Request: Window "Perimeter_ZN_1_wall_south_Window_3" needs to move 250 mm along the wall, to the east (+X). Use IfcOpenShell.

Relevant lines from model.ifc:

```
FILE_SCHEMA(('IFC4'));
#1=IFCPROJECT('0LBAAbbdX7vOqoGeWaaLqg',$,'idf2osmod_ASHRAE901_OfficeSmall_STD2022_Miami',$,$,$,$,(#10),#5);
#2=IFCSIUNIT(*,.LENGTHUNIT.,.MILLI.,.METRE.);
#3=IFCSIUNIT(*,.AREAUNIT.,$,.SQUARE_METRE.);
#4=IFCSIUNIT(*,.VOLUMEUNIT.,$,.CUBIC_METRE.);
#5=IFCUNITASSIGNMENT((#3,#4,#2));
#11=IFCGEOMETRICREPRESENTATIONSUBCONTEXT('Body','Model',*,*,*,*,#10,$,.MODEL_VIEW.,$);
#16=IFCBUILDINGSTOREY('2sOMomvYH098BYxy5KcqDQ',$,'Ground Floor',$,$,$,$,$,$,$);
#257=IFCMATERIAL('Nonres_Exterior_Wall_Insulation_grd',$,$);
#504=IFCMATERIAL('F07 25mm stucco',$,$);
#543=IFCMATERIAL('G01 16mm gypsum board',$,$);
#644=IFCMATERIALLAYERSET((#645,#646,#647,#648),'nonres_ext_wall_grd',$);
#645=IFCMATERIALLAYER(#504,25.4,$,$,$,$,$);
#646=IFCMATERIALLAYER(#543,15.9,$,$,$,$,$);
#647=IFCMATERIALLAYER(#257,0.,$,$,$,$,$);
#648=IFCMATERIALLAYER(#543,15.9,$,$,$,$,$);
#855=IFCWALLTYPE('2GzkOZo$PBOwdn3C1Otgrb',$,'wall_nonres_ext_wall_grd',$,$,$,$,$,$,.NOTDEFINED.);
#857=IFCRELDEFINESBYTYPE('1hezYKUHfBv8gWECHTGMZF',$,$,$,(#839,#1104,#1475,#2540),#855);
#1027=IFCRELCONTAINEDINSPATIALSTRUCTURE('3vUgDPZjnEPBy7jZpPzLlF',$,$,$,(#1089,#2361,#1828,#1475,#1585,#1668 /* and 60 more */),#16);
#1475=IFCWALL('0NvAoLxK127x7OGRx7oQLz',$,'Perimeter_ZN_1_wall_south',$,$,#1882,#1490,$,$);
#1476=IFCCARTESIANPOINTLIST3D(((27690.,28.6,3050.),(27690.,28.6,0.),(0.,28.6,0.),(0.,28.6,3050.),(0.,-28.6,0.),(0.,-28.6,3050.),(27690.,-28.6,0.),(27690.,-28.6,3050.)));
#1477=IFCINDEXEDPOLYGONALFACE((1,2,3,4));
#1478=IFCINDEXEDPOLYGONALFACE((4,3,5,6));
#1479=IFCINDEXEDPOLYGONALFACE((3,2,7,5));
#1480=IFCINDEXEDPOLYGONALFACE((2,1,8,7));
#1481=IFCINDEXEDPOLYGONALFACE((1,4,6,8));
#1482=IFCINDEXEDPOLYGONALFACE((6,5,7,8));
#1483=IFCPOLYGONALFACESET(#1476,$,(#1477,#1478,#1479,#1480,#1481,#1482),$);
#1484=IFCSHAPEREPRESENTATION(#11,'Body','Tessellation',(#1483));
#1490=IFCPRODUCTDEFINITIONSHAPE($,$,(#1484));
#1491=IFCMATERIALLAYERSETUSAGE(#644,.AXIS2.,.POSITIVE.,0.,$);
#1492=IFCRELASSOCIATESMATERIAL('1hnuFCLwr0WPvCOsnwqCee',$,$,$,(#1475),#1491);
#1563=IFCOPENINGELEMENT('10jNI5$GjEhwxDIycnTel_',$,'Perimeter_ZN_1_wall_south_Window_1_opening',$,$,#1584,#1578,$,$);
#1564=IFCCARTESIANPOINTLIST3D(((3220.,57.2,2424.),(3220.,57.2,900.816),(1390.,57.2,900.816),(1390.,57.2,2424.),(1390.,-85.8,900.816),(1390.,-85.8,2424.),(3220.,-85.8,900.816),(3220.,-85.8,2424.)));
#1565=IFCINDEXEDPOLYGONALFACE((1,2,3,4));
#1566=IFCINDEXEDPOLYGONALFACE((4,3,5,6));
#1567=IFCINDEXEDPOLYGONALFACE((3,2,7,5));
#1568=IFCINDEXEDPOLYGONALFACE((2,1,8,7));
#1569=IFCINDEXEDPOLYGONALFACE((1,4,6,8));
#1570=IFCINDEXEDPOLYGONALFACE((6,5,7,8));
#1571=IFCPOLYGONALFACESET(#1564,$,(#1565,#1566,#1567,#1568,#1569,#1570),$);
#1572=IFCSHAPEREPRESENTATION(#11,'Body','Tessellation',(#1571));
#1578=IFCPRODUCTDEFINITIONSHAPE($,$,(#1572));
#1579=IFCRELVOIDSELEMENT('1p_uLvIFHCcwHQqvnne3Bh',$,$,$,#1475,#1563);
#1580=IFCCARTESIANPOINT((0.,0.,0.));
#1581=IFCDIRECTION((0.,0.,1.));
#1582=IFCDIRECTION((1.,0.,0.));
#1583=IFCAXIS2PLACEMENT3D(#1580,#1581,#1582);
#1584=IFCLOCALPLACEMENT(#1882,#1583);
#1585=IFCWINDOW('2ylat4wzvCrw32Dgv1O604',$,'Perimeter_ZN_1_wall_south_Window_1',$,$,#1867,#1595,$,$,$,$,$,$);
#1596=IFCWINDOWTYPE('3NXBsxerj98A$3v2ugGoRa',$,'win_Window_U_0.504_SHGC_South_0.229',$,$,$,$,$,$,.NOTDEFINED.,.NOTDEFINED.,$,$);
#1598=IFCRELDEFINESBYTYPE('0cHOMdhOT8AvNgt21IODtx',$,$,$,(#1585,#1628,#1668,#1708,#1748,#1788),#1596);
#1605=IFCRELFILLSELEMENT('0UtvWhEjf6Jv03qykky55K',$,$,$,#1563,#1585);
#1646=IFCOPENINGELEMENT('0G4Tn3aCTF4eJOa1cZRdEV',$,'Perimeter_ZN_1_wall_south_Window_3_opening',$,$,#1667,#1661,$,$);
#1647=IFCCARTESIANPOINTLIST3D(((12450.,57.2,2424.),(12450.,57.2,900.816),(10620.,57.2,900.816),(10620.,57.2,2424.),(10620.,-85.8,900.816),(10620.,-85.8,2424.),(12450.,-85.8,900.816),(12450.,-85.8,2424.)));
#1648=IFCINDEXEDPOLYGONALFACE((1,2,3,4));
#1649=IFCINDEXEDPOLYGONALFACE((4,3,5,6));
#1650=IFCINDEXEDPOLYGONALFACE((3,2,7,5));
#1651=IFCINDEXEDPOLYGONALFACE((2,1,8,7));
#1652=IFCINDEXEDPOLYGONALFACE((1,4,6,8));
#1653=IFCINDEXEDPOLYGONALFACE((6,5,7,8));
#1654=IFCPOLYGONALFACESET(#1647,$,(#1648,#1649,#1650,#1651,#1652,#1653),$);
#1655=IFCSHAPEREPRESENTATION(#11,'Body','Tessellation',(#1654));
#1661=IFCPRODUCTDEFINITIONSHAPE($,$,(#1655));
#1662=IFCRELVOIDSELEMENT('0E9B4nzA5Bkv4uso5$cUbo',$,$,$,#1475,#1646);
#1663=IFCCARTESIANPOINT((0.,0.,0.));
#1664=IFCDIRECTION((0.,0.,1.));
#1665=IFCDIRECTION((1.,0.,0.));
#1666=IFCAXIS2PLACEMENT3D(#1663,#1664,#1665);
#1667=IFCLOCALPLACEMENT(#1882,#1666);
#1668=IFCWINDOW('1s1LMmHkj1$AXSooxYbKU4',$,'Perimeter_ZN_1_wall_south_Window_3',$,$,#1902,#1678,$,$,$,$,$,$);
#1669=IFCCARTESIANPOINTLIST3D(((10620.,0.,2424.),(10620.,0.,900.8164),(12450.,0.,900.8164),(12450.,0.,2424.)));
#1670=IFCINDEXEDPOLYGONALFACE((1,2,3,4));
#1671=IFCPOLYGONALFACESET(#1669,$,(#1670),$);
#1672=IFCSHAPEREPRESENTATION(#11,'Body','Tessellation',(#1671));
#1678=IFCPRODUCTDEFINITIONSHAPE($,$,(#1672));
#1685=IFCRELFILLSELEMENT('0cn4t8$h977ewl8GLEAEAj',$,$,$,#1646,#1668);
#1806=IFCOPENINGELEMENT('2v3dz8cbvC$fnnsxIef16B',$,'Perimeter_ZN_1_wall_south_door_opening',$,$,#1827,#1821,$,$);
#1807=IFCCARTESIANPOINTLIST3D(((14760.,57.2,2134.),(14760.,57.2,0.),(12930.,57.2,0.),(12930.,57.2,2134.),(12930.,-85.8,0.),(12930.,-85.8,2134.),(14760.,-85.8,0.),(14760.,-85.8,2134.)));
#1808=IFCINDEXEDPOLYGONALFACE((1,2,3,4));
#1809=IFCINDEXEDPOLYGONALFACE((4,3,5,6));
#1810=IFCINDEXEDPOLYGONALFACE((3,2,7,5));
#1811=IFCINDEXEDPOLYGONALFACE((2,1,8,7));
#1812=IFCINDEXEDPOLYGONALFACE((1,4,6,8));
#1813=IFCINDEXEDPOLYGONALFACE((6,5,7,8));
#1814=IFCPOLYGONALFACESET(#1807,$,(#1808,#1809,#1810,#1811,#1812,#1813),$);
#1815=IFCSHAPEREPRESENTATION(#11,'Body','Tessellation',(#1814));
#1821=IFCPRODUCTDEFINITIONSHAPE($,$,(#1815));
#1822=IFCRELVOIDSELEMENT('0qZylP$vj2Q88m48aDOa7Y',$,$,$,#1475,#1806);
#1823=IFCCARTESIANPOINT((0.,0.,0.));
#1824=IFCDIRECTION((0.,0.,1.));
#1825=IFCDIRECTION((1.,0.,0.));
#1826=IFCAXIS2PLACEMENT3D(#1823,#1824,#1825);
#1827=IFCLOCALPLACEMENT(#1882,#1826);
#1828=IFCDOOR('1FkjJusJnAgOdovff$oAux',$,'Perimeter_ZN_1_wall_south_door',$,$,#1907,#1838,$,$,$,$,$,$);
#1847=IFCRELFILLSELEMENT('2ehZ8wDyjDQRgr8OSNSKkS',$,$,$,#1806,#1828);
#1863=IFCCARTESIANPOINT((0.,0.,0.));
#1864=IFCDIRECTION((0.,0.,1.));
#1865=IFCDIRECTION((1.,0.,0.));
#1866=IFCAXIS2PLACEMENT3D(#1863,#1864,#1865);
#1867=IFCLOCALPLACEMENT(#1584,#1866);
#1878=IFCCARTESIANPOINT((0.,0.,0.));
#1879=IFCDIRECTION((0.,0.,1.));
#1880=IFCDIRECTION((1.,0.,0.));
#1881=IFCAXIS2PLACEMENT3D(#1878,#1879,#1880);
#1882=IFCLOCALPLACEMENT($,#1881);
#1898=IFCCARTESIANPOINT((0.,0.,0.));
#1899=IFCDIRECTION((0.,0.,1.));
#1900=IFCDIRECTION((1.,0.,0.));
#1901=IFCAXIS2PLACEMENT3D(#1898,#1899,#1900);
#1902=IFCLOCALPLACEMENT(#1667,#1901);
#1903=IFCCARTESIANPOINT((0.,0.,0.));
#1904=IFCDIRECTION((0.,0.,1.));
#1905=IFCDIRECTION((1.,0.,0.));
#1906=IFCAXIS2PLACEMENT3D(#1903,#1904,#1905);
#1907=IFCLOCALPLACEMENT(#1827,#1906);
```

```python
import ifcopenshell
import ifcopenshell.api.geometry
import ifcopenshell.util.placement

model = ifcopenshell.open("model.ifc")

window = model.by_guid("1s1LMmHkj1$AXSooxYbKU4")
opening = window.FillsVoids[0].RelatingOpeningElement
wall = opening.VoidsElements[0].RelatingBuildingElement

wall_matrix = ifcopenshell.util.placement.get_local_placement(wall.ObjectPlacement)
shift = wall_matrix[:3, 0] * 250.0
before = ifcopenshell.util.placement.get_local_placement(window.ObjectPlacement)[:3, 3].copy()

# The window is placed relative to its opening, so it follows when the opening moves.
matrix = ifcopenshell.util.placement.get_local_placement(opening.ObjectPlacement)
matrix[:3, 3] += shift
ifcopenshell.api.geometry.edit_object_placement(
    model, product=opening, matrix=matrix, is_si=False, should_transform_children=True
)

after = ifcopenshell.util.placement.get_local_placement(window.ObjectPlacement)[:3, 3]
print("window moved by", (after - before).round(3) + 0.0)

model.write("model_edited.ifc")
```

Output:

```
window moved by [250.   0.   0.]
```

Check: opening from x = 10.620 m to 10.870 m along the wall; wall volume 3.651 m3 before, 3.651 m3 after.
